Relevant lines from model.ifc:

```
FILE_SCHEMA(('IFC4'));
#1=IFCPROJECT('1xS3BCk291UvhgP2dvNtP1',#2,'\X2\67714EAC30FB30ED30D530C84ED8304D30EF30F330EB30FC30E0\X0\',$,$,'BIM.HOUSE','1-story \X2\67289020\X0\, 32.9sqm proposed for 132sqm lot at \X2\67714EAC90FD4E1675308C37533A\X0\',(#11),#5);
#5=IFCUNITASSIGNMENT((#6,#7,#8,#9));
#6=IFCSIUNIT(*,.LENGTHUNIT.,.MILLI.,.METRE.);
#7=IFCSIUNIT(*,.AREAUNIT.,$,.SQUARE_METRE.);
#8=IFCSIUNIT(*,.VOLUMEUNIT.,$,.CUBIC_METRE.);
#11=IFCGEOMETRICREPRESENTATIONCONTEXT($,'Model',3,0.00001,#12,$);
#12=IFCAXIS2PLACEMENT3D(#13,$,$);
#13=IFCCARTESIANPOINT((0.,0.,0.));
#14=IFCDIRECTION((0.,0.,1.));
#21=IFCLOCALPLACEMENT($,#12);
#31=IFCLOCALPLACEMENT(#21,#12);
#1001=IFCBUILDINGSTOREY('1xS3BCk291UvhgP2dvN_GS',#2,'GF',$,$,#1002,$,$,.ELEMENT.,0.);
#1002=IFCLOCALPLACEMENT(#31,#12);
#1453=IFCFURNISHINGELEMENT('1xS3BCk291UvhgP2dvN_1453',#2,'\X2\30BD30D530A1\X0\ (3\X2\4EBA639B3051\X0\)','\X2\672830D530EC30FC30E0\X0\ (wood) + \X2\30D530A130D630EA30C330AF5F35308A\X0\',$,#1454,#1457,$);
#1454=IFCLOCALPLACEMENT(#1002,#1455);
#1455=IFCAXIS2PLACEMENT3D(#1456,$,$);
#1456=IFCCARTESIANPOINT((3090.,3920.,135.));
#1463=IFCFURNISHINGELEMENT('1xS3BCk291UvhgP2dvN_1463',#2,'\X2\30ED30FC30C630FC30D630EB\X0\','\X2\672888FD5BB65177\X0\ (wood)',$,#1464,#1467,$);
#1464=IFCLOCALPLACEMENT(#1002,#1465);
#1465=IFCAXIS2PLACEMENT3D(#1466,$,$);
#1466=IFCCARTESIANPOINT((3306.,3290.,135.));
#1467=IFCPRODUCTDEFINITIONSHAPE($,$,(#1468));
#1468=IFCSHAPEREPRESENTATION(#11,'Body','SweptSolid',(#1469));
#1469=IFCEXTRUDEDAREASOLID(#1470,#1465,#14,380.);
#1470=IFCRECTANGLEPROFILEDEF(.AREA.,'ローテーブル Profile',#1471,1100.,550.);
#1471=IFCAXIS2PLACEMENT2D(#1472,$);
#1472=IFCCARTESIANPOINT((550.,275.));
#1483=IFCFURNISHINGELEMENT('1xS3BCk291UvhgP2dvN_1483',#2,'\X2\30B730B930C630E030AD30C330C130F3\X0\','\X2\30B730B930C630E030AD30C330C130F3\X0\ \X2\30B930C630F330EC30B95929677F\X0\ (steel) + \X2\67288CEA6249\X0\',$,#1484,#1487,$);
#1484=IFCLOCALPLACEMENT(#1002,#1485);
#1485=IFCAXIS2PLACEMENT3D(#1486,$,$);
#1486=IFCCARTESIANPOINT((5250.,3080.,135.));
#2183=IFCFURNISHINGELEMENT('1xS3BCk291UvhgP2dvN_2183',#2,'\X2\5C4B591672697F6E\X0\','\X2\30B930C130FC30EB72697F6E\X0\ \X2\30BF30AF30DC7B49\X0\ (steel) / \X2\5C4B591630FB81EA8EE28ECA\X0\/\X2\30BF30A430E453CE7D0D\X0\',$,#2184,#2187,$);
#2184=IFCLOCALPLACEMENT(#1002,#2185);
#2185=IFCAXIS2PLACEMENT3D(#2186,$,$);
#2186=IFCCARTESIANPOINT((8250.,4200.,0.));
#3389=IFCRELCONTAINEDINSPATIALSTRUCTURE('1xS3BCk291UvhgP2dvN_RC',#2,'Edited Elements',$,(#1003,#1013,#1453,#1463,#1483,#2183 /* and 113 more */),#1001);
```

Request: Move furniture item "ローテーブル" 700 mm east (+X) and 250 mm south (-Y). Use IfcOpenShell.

```python
import ifcopenshell
import ifcopenshell.api.geometry
import ifcopenshell.util.placement
import ifcopenshell.util.unit

model = ifcopenshell.open("model.ifc")
unit_scale = ifcopenshell.util.unit.calculate_unit_scale(model)

item = model.by_guid("1xS3BCk291UvhgP2dvN_1463")
matrix = ifcopenshell.util.placement.get_local_placement(item.ObjectPlacement)
matrix[0, 3] += 0.7 / unit_scale
matrix[1, 3] -= 0.25 / unit_scale
ifcopenshell.api.geometry.edit_object_placement(model, product=item, matrix=matrix, is_si=False)

print(ifcopenshell.util.placement.get_local_placement(item.ObjectPlacement).round(3) + 0.0)

model.write("model-out.ifc")
```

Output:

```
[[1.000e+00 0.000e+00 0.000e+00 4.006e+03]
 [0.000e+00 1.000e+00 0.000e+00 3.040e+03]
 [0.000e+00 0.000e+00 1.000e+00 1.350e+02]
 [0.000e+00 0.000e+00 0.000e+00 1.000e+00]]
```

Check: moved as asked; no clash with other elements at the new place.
